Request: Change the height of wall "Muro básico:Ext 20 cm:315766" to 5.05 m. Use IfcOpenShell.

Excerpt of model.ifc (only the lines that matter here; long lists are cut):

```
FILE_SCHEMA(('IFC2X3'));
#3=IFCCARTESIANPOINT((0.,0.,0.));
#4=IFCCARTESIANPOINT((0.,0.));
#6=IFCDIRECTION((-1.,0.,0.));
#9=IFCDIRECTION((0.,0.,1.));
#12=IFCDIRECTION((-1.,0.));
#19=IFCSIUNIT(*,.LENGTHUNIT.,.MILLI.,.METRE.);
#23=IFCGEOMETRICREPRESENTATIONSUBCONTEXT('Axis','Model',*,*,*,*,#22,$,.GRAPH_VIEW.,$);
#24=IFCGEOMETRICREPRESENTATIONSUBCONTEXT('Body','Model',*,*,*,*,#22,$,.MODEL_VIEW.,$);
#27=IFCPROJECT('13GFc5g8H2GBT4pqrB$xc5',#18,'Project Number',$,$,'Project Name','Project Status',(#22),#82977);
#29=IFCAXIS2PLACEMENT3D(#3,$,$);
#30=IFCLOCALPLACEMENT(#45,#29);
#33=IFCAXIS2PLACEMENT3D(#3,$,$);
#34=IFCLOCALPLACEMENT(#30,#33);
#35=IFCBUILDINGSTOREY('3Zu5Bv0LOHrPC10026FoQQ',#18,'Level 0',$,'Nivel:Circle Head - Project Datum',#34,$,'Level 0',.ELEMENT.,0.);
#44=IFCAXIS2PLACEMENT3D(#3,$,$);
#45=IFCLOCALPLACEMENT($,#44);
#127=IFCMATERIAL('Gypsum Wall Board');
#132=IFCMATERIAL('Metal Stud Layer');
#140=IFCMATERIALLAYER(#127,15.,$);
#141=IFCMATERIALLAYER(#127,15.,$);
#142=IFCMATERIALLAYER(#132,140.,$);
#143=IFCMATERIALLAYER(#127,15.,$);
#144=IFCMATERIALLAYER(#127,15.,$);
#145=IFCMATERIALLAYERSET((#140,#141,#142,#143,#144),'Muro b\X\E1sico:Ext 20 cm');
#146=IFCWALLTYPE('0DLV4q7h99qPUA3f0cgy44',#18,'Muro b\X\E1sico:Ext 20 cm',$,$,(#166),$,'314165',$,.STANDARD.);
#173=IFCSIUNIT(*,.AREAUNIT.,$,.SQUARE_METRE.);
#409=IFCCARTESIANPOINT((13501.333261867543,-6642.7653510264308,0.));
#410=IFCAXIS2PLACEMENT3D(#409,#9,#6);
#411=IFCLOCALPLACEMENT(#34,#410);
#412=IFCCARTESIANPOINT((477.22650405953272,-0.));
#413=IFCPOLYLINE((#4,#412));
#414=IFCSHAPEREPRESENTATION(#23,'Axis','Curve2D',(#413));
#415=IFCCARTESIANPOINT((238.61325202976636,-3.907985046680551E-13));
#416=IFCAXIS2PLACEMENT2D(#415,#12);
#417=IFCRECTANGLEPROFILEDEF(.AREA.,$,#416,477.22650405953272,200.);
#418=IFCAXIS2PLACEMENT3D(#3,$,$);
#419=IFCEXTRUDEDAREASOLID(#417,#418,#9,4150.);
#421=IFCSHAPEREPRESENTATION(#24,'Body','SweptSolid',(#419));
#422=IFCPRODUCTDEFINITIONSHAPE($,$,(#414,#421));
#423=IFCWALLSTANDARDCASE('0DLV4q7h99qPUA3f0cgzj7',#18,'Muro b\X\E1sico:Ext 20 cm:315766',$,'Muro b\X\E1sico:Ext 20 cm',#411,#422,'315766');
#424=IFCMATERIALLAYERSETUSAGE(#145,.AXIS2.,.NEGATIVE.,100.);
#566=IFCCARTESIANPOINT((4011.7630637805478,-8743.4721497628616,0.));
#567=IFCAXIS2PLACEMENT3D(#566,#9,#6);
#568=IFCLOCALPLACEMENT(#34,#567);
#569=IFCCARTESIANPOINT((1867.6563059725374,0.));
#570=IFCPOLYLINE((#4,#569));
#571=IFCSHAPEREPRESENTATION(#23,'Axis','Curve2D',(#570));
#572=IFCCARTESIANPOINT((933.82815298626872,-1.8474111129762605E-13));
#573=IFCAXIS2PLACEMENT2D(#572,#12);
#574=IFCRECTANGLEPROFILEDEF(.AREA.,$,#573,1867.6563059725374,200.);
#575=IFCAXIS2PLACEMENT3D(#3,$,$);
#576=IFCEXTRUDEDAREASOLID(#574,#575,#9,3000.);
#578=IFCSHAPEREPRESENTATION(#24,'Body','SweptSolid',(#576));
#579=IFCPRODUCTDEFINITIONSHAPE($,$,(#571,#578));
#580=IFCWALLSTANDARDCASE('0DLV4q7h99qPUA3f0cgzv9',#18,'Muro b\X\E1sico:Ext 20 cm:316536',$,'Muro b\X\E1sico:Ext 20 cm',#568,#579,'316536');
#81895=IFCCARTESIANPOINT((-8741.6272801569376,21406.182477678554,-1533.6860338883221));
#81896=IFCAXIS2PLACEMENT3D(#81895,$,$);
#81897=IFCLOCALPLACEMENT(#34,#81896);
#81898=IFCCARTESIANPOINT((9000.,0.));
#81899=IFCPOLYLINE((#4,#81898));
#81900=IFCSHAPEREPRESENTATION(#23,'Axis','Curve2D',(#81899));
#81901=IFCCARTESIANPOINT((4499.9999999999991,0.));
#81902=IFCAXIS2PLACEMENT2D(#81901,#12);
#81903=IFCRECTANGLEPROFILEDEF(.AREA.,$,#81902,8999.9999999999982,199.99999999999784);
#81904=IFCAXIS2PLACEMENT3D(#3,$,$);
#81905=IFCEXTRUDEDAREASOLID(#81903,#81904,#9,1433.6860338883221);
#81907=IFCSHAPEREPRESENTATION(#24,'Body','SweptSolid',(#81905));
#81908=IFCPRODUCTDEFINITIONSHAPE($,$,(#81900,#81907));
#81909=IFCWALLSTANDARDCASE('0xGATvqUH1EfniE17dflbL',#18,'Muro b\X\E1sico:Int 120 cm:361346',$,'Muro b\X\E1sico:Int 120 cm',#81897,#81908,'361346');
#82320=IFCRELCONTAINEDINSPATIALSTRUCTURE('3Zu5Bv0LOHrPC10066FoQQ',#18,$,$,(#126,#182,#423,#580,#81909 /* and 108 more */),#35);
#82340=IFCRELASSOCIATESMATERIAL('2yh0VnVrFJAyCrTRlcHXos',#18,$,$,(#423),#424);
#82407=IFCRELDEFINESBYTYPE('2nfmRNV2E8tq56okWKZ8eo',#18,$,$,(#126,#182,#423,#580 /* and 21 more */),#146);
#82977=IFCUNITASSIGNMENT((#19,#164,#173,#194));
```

```python
import ifcopenshell
import ifcopenshell.geom
import ifcopenshell.util.representation
import ifcopenshell.util.shape
import ifcopenshell.util.unit

model = ifcopenshell.open("model.ifc")
unit_scale = ifcopenshell.util.unit.calculate_unit_scale(model)
settings = ifcopenshell.geom.settings()


def volume(element):
    """Net volume in cubic metres, openings subtracted."""
    shape = ifcopenshell.geom.create_shape(settings, element)
    return ifcopenshell.util.shape.get_volume(shape.geometry)


wall = model.by_guid("0DLV4q7h99qPUA3f0cgzj7")
before = volume(wall)

body = ifcopenshell.util.representation.get_representation(wall, "Model", "Body")
solid = body.Items[0]
old_height = solid.Depth
solid.Depth = 5.05 / unit_scale
after = volume(wall)

print(f"height {old_height:g} -> {solid.Depth:g}, volume {before:.3f} -> {after:.3f} m3")

model.write("model_v2.ifc")
```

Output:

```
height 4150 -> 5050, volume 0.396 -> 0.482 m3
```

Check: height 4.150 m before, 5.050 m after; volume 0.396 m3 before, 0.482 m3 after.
